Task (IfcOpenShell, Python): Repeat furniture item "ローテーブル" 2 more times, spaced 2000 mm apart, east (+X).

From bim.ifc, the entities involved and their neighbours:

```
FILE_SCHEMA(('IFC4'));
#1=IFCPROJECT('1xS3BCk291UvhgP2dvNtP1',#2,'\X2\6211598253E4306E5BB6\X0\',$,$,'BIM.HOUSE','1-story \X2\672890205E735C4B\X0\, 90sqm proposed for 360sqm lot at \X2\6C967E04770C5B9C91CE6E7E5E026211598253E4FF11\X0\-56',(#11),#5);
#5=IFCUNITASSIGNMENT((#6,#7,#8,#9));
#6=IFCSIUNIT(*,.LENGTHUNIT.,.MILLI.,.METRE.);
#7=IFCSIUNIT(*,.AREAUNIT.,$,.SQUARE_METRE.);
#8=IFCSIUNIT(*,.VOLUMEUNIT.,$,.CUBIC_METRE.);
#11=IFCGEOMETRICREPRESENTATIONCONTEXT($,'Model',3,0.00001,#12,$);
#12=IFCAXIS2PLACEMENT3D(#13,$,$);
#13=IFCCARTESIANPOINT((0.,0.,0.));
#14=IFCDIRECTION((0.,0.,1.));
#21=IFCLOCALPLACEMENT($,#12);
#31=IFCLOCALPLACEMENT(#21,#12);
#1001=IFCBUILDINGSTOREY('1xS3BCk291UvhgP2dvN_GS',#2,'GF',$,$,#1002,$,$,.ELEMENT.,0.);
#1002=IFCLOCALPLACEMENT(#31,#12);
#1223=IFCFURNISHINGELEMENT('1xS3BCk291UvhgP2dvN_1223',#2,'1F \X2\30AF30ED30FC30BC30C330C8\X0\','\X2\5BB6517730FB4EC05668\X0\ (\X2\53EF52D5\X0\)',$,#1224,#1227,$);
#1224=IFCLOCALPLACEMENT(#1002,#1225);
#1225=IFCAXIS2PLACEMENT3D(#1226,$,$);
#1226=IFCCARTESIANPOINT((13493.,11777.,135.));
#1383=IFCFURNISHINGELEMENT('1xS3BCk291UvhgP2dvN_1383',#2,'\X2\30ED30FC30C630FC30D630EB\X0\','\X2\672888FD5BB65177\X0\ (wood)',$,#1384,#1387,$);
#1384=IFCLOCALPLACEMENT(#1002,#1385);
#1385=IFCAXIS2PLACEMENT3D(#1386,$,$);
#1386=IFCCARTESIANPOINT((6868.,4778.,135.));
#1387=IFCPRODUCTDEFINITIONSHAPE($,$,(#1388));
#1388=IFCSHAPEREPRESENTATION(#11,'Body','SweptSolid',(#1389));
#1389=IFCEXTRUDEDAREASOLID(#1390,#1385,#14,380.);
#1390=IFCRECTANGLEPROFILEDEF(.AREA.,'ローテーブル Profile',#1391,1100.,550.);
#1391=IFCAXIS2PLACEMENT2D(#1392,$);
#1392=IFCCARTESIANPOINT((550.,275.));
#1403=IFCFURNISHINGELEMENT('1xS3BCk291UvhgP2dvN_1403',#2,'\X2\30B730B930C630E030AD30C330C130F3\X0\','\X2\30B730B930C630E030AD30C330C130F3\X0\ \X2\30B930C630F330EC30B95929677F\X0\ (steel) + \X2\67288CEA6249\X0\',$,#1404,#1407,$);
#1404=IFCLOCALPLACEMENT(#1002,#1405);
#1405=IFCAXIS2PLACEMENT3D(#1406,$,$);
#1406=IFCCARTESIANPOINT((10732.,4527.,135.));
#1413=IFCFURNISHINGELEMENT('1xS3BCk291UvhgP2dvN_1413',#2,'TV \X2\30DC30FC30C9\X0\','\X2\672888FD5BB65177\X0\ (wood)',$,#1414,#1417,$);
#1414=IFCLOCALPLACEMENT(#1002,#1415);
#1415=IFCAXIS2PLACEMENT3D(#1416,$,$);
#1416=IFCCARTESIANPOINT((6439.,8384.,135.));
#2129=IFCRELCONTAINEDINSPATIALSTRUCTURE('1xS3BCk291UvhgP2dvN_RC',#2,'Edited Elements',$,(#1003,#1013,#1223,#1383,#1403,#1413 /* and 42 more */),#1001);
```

```python
import numpy as np
import ifcopenshell
import ifcopenshell.api.geometry
import ifcopenshell.api.root
import ifcopenshell.util.element
import ifcopenshell.util.placement
import ifcopenshell.util.unit

model = ifcopenshell.open("bim.ifc")
unit_scale = ifcopenshell.util.unit.calculate_unit_scale(model)


def reuse_history(source, copy):
    """copy_class also copies each property set's owner history, people and application; keep the originals."""
    for rel in copy.IsDefinedBy:
        if rel.is_a("IfcRelDefinesByProperties") and (history := rel.RelatingPropertyDefinition.OwnerHistory):
            rel.RelatingPropertyDefinition.OwnerHistory = source.OwnerHistory
            ifcopenshell.util.element.remove_deep2(model, history)


source = model.by_guid("1xS3BCk291UvhgP2dvN_1383")
base = ifcopenshell.util.placement.get_local_placement(source.ObjectPlacement)
step = np.array([1.0, 0.0, 0.0]) * 2 / unit_scale

for i in range(1, 3):
    copy = ifcopenshell.api.root.copy_class(model, product=source)
    copy.Representation = ifcopenshell.util.element.copy_deep(
        model, source.Representation, exclude=["IfcGeometricRepresentationContext", "IfcRepresentationMap"]
    )
    reuse_history(source, copy)
    matrix = base.copy()
    matrix[:3, 3] += i * step
    print("added at", matrix[:3, 3].round(3) + 0.0)
    ifcopenshell.api.geometry.edit_object_placement(model, product=copy, matrix=matrix, is_si=False)

model.write("bim_updated.ifc")
```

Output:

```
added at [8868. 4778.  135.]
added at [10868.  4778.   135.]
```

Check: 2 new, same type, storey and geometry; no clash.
